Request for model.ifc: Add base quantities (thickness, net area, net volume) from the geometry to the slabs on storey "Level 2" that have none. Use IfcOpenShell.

First a look at what the model holds.

```python
import ifcopenshell
import ifcopenshell.util.element
import ifcopenshell.util.unit

model = ifcopenshell.open("model.ifc")
print(model.schema)
for unit_type in ("LENGTHUNIT", "AREAUNIT", "VOLUMEUNIT"):
    print(unit_type, ifcopenshell.util.unit.calculate_unit_scale(model, unit_type))
storey = next(s for s in model.by_type("IfcBuildingStorey") if s.Name == "Level 2")
slabs = [e for e in ifcopenshell.util.element.get_decomposition(storey) if e.is_a("IfcSlab")]
for e in sorted(slabs, key=lambda e: e.id()):
    print(e.id(), e.is_a(), e.Name, list(ifcopenshell.util.element.get_psets(e, qtos_only=True)), sep=" | ")
```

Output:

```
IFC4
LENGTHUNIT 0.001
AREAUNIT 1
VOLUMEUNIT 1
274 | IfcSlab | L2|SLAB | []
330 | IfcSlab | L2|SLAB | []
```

```python
import ifcopenshell
import ifcopenshell.api.pset
import ifcopenshell.geom
import ifcopenshell.util.element
import ifcopenshell.util.shape
import ifcopenshell.util.unit

model = ifcopenshell.open("model.ifc")
unit_scale = ifcopenshell.util.unit.calculate_unit_scale(model)
area_scale = ifcopenshell.util.unit.calculate_unit_scale(model, "AREAUNIT")
volume_scale = ifcopenshell.util.unit.calculate_unit_scale(model, "VOLUMEUNIT")
settings = ifcopenshell.geom.settings()

storey = next(s for s in model.by_type("IfcBuildingStorey") if s.Name == "Level 2")
slabs = [e for e in ifcopenshell.util.element.get_decomposition(storey) if e.is_a("IfcSlab")]

for e in sorted(slabs, key=lambda e: e.id()):
    if ifcopenshell.util.element.get_psets(e, qtos_only=True, should_inherit=False):
        continue
    # Geometry comes back in metres, in the element's own axes.
    shape = ifcopenshell.geom.create_shape(settings, e)
    values = {
        "Width": ifcopenshell.util.shape.get_z(shape.geometry) / unit_scale,
        "NetArea": ifcopenshell.util.shape.get_footprint_area(shape.geometry) / area_scale,
        "NetVolume": ifcopenshell.util.shape.get_volume(shape.geometry) / volume_scale,
    }
    qto = ifcopenshell.api.pset.add_qto(model, product=e, name="Qto_SlabBaseQuantities")
    ifcopenshell.api.pset.edit_qto(model, qto=qto, properties=values)
    print(e.id(), {k: round(v, 3) for k, v in values.items()})

model.write("model_edited.ifc")
```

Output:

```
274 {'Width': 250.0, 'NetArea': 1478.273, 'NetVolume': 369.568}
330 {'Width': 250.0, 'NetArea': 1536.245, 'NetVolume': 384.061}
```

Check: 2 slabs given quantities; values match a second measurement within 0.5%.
